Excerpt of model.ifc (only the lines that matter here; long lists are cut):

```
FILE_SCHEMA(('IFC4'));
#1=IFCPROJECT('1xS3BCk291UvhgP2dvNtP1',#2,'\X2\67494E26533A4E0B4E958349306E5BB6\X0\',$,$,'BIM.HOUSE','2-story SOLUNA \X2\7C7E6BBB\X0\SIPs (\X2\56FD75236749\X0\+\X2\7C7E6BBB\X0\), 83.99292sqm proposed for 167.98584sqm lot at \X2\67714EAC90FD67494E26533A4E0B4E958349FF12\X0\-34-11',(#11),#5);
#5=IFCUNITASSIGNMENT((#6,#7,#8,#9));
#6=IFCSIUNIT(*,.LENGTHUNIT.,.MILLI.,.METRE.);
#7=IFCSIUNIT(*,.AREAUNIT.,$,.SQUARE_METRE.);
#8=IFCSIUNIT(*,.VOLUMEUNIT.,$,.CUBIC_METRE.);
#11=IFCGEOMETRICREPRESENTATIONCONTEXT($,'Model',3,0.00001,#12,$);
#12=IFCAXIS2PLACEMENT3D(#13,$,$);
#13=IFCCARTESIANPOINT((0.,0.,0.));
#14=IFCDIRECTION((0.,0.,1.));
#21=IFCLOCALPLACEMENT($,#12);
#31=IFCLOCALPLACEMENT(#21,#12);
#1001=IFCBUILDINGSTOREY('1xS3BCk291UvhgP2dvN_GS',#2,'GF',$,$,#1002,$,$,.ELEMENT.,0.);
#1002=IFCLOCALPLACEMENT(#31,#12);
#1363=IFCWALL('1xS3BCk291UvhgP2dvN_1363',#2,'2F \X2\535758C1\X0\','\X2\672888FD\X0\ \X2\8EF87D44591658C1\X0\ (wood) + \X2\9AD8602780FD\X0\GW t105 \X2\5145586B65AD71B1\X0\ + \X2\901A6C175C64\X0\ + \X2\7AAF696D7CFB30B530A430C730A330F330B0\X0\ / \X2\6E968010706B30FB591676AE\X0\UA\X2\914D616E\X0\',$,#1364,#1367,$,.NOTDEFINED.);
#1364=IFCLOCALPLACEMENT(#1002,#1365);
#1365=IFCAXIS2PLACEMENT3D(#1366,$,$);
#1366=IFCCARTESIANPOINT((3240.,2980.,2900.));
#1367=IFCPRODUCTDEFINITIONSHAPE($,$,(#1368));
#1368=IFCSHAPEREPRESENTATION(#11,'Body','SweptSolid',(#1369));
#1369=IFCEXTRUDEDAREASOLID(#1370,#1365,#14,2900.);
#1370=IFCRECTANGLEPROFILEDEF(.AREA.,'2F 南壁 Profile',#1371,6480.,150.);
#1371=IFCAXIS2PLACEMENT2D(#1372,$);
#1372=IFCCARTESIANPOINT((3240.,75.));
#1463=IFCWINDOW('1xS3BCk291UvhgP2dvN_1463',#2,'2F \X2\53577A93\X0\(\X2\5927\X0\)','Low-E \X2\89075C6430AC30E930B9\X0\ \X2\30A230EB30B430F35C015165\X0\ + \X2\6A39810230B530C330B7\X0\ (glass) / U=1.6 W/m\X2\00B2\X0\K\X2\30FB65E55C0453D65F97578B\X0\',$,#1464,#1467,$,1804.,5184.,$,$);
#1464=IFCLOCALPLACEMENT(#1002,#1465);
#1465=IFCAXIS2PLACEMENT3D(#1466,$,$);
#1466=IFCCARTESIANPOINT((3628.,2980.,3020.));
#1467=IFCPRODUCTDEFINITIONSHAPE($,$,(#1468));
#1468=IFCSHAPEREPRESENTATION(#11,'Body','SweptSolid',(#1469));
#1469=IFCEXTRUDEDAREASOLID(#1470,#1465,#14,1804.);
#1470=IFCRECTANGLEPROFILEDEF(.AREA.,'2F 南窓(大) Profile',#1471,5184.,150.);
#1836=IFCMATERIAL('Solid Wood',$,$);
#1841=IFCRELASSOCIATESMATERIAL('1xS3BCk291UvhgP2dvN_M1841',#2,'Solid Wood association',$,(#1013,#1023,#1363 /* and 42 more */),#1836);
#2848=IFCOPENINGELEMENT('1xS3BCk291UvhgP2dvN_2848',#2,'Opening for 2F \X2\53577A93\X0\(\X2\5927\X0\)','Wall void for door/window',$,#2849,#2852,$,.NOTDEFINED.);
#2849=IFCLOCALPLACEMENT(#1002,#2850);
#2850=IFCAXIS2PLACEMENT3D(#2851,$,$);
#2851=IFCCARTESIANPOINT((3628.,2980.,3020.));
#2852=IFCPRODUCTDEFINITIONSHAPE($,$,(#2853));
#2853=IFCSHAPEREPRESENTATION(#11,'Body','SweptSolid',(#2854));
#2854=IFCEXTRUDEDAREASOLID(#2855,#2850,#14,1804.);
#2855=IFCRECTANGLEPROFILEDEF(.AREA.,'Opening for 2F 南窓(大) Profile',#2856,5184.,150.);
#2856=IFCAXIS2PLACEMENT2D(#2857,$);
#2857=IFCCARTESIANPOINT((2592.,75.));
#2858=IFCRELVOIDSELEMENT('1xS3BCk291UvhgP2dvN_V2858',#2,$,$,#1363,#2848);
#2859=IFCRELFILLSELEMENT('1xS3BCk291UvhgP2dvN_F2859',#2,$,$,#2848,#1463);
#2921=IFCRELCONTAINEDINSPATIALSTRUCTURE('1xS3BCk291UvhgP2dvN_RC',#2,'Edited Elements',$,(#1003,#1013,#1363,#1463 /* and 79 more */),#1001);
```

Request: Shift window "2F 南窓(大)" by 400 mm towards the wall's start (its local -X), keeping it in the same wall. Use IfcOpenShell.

```python
import ifcopenshell
import ifcopenshell.api.geometry
import ifcopenshell.util.placement

model = ifcopenshell.open("model.ifc")

window = model.by_guid("1xS3BCk291UvhgP2dvN_1463")
opening = window.FillsVoids[0].RelatingOpeningElement
wall = opening.VoidsElements[0].RelatingBuildingElement

wall_matrix = ifcopenshell.util.placement.get_local_placement(wall.ObjectPlacement)
shift = wall_matrix[:3, 0] * -400.0
before = ifcopenshell.util.placement.get_local_placement(window.ObjectPlacement)[:3, 3].copy()

# The window is not placed relative to its opening, so move both.
for product in (opening, window):
    matrix = ifcopenshell.util.placement.get_local_placement(product.ObjectPlacement)
    matrix[:3, 3] += shift
    ifcopenshell.api.geometry.edit_object_placement(model, product=product, matrix=matrix, is_si=False)

after = ifcopenshell.util.placement.get_local_placement(window.ObjectPlacement)[:3, 3]
print("window moved by", (after - before).round(3) + 0.0)

model.write("model_edited.ifc")
```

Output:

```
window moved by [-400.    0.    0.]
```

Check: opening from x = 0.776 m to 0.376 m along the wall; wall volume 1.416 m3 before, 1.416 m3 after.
